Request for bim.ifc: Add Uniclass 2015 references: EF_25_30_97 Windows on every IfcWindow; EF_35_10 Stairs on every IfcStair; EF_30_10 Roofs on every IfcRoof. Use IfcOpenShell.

First a look at what the model holds.

```python
import ifcopenshell

model = ifcopenshell.open("bim.ifc")
print(model.schema)
print("classifications:", [c.Name for c in model.by_type("IfcClassification")])
for ifc_class in ("IfcDoor", "IfcRoof", "IfcStair", "IfcWall", "IfcWindow"):
    print(ifc_class, len(model.by_type(ifc_class)))
```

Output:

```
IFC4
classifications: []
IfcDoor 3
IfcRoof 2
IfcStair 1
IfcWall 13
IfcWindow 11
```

```python
import ifcopenshell
import ifcopenshell.api.classification

model = ifcopenshell.open("bim.ifc")

system = ifcopenshell.api.classification.add_classification(model, classification="Uniclass 2015")

codes = {
    "IfcWindow": ("EF_25_30_97", "Windows"),
    "IfcStair": ("EF_35_10", "Stairs"),
    "IfcRoof": ("EF_30_10", "Roofs"),
}
for ifc_class, (code, name) in codes.items():
    products = model.by_type(ifc_class)
    ifcopenshell.api.classification.add_reference(
        model, products=products, classification=system, identification=code, name=name
    )
    print(code, len(products))

model.write("bim_rev.ifc")
```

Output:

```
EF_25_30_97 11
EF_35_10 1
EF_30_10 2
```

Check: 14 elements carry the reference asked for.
